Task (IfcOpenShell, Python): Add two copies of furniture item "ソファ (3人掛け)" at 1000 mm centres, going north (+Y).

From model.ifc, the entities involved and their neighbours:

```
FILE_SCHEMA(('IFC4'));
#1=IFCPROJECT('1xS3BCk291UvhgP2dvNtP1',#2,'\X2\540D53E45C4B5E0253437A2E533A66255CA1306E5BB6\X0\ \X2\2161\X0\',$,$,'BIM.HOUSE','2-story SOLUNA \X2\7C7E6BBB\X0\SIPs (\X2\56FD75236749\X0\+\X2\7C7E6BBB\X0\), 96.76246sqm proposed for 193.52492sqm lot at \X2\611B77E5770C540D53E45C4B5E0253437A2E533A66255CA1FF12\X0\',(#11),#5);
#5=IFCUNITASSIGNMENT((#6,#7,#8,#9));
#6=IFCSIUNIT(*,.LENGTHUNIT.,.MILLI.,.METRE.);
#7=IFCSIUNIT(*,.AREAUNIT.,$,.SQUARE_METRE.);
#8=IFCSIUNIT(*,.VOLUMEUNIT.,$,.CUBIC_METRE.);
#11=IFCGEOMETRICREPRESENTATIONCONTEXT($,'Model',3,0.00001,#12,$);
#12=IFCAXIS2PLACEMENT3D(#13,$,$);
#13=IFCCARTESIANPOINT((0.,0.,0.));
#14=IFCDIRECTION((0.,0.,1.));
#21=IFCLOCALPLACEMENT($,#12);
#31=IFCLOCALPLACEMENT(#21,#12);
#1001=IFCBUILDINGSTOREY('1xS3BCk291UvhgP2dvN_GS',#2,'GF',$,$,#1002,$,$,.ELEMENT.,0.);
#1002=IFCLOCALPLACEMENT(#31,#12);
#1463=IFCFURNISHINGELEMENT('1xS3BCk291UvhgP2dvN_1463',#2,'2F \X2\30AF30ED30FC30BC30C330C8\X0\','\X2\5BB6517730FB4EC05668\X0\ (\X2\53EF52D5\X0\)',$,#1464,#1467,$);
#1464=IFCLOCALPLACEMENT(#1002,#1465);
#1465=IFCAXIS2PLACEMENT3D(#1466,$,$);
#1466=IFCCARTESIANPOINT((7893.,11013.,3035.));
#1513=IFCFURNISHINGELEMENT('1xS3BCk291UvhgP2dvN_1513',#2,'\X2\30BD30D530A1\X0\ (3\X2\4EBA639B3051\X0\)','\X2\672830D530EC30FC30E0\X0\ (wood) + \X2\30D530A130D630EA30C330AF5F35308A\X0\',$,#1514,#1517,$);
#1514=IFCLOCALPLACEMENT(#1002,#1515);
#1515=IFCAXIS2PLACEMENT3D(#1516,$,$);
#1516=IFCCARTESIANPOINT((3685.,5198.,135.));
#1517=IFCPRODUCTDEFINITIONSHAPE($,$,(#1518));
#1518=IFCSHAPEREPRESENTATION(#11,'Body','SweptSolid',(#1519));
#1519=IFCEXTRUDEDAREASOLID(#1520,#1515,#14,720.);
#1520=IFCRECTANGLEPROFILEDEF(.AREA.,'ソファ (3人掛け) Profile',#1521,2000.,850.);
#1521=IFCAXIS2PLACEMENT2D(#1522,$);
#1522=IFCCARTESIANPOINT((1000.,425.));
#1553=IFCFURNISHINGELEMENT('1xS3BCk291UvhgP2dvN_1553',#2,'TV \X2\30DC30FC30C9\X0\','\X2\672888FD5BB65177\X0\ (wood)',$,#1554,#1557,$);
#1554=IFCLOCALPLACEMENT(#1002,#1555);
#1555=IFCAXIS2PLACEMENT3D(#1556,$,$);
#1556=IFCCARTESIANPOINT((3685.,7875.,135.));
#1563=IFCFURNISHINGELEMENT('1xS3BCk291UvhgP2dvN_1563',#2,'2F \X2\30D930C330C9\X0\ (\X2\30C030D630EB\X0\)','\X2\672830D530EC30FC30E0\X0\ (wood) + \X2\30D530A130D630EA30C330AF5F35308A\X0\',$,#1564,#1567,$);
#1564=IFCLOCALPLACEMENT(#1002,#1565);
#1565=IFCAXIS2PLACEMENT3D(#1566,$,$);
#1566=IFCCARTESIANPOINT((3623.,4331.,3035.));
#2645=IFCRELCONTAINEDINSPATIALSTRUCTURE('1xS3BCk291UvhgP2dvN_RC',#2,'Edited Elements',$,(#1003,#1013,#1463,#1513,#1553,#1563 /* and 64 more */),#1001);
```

```python
import numpy as np
import ifcopenshell
import ifcopenshell.api.geometry
import ifcopenshell.api.root
import ifcopenshell.util.element
import ifcopenshell.util.placement
import ifcopenshell.util.unit

model = ifcopenshell.open("model.ifc")
unit_scale = ifcopenshell.util.unit.calculate_unit_scale(model)


def reuse_history(source, copy):
    """copy_class also copies each property set's owner history, people and application; keep the originals."""
    for rel in copy.IsDefinedBy:
        if rel.is_a("IfcRelDefinesByProperties") and (history := rel.RelatingPropertyDefinition.OwnerHistory):
            rel.RelatingPropertyDefinition.OwnerHistory = source.OwnerHistory
            ifcopenshell.util.element.remove_deep2(model, history)


source = model.by_id(1513)
base = ifcopenshell.util.placement.get_local_placement(source.ObjectPlacement)
step = np.array([0.0, 1.0, 0.0]) * 1 / unit_scale

for i in range(1, 3):
    copy = ifcopenshell.api.root.copy_class(model, product=source)
    copy.Representation = ifcopenshell.util.element.copy_deep(
        model, source.Representation, exclude=["IfcGeometricRepresentationContext", "IfcRepresentationMap"]
    )
    reuse_history(source, copy)
    matrix = base.copy()
    matrix[:3, 3] += i * step
    print("added at", matrix[:3, 3].round(3) + 0.0)
    ifcopenshell.api.geometry.edit_object_placement(model, product=copy, matrix=matrix, is_si=False)

model.write("model_updated.ifc")
```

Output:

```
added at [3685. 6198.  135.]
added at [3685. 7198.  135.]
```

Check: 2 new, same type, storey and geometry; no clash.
